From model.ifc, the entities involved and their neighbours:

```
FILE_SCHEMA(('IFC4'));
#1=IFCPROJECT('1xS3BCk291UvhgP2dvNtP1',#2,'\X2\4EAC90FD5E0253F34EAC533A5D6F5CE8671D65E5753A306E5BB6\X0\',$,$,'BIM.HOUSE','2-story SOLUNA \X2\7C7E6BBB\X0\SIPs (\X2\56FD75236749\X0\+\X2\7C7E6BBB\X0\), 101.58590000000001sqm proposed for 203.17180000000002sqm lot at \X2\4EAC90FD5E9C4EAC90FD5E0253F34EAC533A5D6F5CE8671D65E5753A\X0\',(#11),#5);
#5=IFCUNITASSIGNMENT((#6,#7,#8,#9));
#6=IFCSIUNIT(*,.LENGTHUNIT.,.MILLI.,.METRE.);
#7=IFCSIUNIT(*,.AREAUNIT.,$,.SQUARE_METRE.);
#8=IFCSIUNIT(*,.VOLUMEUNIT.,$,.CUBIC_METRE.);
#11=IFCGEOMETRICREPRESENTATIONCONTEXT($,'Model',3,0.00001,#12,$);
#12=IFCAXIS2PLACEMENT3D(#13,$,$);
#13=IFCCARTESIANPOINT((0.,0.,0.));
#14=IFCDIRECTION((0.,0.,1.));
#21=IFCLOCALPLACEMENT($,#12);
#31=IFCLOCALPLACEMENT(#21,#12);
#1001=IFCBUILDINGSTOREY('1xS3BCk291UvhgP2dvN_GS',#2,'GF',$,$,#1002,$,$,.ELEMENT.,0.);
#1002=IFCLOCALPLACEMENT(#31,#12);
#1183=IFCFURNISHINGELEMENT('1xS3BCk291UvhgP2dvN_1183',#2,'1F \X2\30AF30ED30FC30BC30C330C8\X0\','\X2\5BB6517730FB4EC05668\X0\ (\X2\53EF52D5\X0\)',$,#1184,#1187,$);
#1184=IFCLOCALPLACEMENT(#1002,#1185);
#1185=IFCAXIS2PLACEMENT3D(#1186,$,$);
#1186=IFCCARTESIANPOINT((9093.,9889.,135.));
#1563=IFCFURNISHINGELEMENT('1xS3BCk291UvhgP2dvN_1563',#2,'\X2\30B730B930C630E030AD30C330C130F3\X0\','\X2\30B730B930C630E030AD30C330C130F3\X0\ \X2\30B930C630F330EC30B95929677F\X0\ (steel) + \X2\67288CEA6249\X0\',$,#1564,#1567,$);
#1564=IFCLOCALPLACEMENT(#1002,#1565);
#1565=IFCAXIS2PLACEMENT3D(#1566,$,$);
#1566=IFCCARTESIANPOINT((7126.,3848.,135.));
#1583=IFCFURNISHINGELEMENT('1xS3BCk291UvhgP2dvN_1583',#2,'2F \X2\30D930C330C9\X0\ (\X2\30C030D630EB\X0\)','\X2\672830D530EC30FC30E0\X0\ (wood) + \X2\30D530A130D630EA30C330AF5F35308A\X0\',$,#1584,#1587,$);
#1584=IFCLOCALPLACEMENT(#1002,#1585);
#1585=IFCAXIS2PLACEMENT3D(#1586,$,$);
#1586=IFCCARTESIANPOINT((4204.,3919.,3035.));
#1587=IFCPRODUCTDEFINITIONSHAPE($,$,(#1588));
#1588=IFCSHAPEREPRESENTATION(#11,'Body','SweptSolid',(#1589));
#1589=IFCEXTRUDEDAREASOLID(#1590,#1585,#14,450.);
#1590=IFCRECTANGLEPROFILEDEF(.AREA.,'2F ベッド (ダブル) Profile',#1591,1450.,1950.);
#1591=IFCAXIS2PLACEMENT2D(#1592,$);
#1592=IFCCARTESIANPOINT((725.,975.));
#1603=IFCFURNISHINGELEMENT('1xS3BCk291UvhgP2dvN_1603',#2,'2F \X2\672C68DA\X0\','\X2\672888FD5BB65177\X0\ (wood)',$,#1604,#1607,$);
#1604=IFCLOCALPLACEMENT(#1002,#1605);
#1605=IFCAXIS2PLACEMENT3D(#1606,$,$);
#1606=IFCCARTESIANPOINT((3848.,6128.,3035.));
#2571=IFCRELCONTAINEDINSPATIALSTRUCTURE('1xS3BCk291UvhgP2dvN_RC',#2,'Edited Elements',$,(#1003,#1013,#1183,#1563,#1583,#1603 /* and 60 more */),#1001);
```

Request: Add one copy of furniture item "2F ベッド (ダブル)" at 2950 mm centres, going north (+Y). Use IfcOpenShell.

```python
import numpy as np
import ifcopenshell
import ifcopenshell.api.geometry
import ifcopenshell.api.root
import ifcopenshell.util.element
import ifcopenshell.util.placement
import ifcopenshell.util.unit

model = ifcopenshell.open("model.ifc")
unit_scale = ifcopenshell.util.unit.calculate_unit_scale(model)


def reuse_history(source, copy):
    """copy_class also copies each property set's owner history, people and application; keep the originals."""
    for rel in copy.IsDefinedBy:
        if rel.is_a("IfcRelDefinesByProperties") and (history := rel.RelatingPropertyDefinition.OwnerHistory):
            rel.RelatingPropertyDefinition.OwnerHistory = source.OwnerHistory
            ifcopenshell.util.element.remove_deep2(model, history)


source = model.by_guid("1xS3BCk291UvhgP2dvN_1583")
base = ifcopenshell.util.placement.get_local_placement(source.ObjectPlacement)
step = np.array([0.0, 1.0, 0.0]) * 2.95 / unit_scale

for i in range(1, 2):
    copy = ifcopenshell.api.root.copy_class(model, product=source)
    copy.Representation = ifcopenshell.util.element.copy_deep(
        model, source.Representation, exclude=["IfcGeometricRepresentationContext", "IfcRepresentationMap"]
    )
    reuse_history(source, copy)
    matrix = base.copy()
    matrix[:3, 3] += i * step
    print("added at", matrix[:3, 3].round(3) + 0.0)
    ifcopenshell.api.geometry.edit_object_placement(model, product=copy, matrix=matrix, is_si=False)

model.write("model_updated.ifc")
```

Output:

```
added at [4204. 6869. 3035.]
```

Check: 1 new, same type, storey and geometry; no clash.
